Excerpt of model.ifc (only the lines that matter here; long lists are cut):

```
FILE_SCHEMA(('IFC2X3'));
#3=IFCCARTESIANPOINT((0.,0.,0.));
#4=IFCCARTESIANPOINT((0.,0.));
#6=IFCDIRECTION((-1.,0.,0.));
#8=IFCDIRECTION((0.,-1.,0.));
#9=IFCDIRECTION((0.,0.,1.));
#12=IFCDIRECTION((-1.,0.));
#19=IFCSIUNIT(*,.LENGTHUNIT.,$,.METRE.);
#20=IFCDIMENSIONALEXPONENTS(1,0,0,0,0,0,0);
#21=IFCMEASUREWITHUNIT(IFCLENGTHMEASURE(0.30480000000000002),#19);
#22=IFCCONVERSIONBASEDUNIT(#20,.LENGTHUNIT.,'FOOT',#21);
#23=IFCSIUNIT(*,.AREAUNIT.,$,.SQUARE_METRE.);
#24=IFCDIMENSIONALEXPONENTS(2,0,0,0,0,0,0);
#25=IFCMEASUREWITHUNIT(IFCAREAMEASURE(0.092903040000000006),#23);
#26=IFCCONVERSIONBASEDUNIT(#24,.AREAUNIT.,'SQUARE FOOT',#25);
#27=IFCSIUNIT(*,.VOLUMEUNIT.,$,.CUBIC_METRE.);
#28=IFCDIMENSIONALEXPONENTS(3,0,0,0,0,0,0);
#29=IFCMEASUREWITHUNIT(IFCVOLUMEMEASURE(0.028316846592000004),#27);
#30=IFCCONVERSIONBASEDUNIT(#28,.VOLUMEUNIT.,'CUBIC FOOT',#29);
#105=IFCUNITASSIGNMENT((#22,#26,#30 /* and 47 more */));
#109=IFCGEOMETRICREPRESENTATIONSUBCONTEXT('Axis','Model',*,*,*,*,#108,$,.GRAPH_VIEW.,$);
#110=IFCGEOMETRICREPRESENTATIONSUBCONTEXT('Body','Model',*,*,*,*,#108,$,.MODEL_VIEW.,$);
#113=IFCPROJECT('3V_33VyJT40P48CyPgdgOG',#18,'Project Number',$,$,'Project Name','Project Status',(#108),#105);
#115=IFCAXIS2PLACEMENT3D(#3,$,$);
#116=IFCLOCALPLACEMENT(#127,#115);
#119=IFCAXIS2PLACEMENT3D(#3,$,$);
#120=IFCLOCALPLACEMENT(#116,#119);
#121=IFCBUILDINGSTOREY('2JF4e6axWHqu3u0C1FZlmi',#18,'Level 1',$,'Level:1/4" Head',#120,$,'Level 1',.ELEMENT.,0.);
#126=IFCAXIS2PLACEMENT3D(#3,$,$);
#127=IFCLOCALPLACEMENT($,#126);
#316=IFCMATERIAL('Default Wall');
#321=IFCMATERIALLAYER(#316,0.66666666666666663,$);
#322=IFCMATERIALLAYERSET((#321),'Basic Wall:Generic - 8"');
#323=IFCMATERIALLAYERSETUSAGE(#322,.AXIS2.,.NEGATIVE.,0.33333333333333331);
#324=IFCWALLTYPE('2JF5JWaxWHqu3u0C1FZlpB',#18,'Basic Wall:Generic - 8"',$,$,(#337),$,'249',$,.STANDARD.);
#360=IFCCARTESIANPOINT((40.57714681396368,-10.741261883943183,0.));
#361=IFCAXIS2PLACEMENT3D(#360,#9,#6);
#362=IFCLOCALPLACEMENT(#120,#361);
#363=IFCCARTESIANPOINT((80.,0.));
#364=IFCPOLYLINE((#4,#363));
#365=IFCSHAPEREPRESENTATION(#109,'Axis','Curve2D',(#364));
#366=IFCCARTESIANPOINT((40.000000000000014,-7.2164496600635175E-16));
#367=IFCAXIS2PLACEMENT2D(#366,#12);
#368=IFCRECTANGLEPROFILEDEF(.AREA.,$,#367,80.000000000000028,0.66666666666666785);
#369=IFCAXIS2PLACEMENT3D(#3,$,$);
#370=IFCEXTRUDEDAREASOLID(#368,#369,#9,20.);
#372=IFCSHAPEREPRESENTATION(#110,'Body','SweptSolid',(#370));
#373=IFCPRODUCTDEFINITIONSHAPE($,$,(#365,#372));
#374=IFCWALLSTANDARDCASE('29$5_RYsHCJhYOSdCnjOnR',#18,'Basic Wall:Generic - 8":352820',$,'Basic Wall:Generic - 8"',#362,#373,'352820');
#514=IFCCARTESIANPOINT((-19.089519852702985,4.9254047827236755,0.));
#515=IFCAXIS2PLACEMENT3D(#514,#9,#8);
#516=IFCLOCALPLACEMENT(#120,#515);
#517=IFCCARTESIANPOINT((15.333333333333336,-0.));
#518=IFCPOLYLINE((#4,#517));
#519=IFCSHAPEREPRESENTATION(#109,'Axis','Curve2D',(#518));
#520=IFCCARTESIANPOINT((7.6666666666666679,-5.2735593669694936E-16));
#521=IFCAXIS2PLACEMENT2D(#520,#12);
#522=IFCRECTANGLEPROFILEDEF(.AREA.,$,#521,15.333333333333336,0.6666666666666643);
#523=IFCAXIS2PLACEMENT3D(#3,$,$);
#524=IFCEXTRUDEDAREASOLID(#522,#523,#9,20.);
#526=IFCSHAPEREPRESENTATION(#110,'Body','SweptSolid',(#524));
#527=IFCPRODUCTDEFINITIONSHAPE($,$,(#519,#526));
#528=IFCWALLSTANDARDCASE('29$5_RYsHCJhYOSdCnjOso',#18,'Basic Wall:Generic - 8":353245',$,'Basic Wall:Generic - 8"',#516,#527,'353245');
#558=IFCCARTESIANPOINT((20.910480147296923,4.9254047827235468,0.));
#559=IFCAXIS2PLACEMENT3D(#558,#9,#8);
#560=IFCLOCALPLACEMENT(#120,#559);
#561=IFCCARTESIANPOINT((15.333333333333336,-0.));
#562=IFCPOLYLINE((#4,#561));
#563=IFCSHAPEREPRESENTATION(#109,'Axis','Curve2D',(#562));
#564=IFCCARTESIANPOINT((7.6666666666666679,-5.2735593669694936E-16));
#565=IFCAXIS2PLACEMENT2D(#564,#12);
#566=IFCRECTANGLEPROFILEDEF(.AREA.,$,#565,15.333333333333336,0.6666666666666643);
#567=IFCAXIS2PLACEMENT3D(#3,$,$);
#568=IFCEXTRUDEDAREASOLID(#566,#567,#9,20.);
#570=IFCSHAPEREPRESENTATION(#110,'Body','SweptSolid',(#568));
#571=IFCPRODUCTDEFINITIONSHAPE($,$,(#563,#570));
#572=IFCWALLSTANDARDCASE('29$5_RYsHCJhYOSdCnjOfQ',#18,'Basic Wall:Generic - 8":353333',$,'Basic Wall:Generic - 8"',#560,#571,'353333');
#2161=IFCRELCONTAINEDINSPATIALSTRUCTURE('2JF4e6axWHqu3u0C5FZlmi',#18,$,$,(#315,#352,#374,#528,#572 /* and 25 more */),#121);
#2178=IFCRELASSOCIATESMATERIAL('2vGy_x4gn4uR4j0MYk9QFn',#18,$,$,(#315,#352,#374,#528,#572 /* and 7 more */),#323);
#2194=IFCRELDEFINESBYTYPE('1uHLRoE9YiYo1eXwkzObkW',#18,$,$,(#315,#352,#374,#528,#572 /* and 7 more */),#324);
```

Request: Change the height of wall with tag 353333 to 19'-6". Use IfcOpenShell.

```python
import ifcopenshell
import ifcopenshell.geom
import ifcopenshell.util.representation
import ifcopenshell.util.shape
import ifcopenshell.util.unit

model = ifcopenshell.open("model.ifc")
unit_scale = ifcopenshell.util.unit.calculate_unit_scale(model)
settings = ifcopenshell.geom.settings()


def volume(element):
    """Net volume in cubic metres, openings subtracted."""
    shape = ifcopenshell.geom.create_shape(settings, element)
    return ifcopenshell.util.shape.get_volume(shape.geometry)


wall = model.by_guid("29$5_RYsHCJhYOSdCnjOfQ")
before = volume(wall)

body = ifcopenshell.util.representation.get_representation(wall, "Model", "Body")
solid = body.Items[0]
old_height = solid.Depth
solid.Depth = 234 * 0.0254 / unit_scale
after = volume(wall)

print(f"height {old_height:g} -> {solid.Depth:g}, volume {before:.3f} -> {after:.3f} m3")

model.write("model_updated.ifc")
```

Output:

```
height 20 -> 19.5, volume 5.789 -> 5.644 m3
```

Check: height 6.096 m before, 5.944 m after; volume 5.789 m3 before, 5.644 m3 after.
